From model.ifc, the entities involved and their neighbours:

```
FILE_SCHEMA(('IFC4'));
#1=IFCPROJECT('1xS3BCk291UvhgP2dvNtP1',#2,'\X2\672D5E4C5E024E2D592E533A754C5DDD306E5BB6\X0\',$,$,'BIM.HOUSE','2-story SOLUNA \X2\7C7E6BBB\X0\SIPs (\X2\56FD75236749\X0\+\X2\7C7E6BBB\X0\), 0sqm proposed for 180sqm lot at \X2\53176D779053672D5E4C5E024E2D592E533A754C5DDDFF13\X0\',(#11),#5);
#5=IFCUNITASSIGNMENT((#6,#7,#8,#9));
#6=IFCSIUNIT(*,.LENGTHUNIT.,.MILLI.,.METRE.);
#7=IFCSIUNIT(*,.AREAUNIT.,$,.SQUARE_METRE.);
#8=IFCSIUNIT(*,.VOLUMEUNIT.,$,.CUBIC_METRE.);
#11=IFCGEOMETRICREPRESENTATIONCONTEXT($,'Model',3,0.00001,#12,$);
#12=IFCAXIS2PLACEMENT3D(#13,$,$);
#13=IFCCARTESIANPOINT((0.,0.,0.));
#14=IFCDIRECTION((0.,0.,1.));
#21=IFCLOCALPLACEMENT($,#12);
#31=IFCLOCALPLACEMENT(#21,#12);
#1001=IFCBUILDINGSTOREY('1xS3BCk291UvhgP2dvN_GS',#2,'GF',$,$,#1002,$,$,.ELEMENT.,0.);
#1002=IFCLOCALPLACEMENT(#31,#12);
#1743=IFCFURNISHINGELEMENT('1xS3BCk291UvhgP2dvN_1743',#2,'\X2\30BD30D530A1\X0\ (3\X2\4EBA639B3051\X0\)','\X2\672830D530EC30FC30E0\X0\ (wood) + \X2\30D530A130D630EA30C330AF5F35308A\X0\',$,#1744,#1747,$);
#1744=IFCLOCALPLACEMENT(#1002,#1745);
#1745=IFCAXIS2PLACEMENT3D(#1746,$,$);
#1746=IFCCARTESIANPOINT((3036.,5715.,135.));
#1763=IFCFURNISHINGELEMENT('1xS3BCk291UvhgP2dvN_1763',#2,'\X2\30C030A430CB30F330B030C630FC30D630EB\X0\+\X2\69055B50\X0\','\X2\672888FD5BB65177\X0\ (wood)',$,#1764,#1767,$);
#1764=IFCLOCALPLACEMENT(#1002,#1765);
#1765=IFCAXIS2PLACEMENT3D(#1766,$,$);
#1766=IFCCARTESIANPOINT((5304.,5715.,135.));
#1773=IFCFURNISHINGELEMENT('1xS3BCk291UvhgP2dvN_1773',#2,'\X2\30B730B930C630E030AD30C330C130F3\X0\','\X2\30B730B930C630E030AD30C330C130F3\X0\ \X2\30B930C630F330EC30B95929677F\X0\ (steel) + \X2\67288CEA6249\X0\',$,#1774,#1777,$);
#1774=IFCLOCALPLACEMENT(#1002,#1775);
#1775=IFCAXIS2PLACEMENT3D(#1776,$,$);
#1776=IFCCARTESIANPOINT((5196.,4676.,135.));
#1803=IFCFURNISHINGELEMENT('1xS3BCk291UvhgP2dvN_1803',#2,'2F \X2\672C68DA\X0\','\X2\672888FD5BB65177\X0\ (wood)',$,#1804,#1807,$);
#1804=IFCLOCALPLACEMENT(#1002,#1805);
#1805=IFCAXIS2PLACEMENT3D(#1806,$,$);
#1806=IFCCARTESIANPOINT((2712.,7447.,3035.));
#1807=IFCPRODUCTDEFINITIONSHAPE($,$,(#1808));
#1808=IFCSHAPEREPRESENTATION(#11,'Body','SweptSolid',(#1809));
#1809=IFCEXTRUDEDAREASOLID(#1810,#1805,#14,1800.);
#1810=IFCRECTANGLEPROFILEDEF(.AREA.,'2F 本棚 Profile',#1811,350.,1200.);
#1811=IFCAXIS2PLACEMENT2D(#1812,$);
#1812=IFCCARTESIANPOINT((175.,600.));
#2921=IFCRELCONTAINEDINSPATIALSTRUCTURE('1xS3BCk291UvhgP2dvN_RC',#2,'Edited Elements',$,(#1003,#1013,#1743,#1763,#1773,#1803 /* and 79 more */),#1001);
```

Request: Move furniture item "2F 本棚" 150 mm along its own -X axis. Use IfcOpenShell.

```python
import ifcopenshell
import ifcopenshell.api.geometry
import ifcopenshell.util.placement
import ifcopenshell.util.unit

model = ifcopenshell.open("model.ifc")
unit_scale = ifcopenshell.util.unit.calculate_unit_scale(model)

item = model.by_id(1803)
matrix = ifcopenshell.util.placement.get_local_placement(item.ObjectPlacement)
matrix[:3, 3] -= matrix[:3, 0] * 0.15 / unit_scale
ifcopenshell.api.geometry.edit_object_placement(model, product=item, matrix=matrix, is_si=False)

print(ifcopenshell.util.placement.get_local_placement(item.ObjectPlacement).round(3) + 0.0)

model.write("model_v2.ifc")
```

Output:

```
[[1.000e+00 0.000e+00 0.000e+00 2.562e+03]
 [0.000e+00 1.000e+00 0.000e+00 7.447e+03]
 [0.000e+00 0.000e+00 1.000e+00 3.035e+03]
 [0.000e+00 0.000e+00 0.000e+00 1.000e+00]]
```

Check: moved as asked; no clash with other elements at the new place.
